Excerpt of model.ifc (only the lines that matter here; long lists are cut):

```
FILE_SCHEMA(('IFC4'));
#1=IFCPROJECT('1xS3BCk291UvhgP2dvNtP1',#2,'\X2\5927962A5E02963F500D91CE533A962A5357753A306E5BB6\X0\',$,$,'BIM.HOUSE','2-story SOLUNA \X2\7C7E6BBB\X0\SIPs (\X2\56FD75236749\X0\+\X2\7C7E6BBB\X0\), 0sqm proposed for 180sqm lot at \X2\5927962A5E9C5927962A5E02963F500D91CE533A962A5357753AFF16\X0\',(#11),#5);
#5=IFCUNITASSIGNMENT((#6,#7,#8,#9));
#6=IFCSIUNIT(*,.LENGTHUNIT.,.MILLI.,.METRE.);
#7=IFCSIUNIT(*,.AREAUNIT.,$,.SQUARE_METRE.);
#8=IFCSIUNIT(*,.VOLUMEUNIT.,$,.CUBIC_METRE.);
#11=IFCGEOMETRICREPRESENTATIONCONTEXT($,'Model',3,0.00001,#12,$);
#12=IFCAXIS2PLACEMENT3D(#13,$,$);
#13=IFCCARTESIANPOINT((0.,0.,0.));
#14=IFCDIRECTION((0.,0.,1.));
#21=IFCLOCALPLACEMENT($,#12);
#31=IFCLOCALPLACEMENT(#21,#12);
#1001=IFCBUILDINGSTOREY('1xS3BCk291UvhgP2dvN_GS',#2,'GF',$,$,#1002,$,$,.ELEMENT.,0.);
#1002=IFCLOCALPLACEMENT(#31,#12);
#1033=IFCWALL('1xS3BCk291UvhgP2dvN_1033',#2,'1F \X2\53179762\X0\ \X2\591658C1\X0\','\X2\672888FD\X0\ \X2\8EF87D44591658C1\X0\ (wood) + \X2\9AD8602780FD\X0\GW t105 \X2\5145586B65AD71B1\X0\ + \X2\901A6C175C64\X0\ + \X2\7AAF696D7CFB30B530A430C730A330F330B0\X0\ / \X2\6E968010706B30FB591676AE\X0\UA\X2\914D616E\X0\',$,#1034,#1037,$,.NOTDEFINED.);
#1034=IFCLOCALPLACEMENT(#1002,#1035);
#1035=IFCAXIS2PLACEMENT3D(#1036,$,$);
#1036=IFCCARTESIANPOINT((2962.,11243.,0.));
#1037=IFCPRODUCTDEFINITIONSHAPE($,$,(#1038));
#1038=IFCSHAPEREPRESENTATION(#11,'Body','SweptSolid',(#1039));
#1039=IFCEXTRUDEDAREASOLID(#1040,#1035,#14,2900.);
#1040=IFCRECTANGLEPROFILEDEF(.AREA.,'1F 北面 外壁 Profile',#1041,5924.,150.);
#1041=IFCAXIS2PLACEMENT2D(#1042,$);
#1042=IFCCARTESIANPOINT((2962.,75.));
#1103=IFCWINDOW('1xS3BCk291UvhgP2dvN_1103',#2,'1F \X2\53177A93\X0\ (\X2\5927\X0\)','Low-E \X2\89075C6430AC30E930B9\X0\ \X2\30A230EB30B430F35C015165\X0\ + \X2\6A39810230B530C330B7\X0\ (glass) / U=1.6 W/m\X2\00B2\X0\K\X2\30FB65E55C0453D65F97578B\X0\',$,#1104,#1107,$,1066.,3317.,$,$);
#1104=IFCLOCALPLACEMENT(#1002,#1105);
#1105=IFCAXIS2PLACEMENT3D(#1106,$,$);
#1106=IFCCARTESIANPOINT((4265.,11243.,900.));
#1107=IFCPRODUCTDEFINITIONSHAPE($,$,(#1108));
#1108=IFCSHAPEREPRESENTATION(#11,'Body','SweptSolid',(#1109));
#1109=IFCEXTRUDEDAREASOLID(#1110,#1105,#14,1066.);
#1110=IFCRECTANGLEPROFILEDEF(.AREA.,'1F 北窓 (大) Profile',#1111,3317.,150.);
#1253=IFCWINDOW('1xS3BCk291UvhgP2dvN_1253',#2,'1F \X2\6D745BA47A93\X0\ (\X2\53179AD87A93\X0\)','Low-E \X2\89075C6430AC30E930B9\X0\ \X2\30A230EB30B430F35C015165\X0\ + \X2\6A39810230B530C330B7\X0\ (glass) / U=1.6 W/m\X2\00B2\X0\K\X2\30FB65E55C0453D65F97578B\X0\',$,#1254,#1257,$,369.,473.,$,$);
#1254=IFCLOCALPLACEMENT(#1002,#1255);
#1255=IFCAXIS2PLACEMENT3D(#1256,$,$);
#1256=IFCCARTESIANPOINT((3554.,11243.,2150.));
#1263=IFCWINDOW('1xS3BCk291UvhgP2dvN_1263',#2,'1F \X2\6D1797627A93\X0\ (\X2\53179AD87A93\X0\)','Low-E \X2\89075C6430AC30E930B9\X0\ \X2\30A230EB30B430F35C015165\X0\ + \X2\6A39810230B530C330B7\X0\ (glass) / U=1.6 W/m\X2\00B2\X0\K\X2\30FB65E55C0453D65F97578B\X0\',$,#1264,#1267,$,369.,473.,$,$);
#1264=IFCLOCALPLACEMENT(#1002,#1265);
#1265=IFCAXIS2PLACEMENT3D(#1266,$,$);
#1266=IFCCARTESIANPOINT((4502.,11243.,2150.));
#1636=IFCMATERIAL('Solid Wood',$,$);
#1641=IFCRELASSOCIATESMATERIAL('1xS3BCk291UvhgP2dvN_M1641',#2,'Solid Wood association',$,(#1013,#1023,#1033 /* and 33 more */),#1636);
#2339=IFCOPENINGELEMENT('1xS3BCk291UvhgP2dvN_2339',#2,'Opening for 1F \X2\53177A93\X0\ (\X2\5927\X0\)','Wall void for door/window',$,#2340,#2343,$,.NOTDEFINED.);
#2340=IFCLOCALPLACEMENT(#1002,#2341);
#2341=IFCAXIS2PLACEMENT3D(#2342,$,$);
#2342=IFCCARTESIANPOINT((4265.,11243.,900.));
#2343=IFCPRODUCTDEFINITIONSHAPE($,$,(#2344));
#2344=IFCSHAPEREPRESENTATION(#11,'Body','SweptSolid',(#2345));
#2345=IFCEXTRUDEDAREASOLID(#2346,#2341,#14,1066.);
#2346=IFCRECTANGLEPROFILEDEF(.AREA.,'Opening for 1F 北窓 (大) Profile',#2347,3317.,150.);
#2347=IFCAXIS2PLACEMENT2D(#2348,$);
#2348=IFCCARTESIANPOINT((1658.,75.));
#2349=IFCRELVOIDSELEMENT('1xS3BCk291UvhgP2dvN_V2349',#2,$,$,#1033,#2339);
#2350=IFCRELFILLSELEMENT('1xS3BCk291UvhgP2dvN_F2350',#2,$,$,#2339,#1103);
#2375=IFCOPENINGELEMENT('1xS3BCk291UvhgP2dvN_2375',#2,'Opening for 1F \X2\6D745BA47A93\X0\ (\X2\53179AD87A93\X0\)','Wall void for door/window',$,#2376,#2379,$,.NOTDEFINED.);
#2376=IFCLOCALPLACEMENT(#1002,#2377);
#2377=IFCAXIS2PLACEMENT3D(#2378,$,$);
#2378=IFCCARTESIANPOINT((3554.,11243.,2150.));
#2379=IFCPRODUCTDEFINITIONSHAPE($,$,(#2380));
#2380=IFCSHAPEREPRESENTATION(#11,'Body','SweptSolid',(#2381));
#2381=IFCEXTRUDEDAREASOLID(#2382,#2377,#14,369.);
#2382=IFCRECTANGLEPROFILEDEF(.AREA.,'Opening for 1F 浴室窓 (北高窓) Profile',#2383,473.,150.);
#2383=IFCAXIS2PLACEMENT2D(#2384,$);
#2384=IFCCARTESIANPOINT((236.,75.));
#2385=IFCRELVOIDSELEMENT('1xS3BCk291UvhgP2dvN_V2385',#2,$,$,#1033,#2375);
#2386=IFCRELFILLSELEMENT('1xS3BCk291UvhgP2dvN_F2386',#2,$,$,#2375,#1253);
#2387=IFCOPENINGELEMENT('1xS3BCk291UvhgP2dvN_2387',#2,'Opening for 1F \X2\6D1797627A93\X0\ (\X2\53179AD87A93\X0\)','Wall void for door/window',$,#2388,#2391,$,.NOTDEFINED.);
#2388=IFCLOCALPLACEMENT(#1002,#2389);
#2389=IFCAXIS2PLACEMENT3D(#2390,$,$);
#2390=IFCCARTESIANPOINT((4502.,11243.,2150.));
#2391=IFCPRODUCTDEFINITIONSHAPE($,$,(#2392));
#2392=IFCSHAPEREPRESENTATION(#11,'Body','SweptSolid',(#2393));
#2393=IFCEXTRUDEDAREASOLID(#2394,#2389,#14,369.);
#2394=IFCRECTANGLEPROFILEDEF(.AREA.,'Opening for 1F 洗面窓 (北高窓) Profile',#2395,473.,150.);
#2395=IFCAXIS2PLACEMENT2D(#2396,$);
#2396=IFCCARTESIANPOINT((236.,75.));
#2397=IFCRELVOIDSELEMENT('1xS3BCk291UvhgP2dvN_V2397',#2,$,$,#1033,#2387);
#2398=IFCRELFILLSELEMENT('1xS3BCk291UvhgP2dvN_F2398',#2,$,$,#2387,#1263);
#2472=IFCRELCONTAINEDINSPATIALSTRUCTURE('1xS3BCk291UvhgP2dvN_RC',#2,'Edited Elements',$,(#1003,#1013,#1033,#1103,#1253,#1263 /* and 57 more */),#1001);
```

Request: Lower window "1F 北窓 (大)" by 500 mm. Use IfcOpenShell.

```python
import numpy as np
import ifcopenshell
import ifcopenshell.api.geometry
import ifcopenshell.util.placement
import ifcopenshell.util.unit

model = ifcopenshell.open("model.ifc")
unit_scale = ifcopenshell.util.unit.calculate_unit_scale(model)

window = model.by_guid("1xS3BCk291UvhgP2dvN_1103")
opening = window.FillsVoids[0].RelatingOpeningElement
dz = -0.5 / unit_scale

shift = np.array([0.0, 0.0, dz])
# The window is not placed relative to its opening, so move both.
for product in (opening, window):
    matrix = ifcopenshell.util.placement.get_local_placement(product.ObjectPlacement)
    matrix[:3, 3] += shift
    ifcopenshell.api.geometry.edit_object_placement(model, product=product, matrix=matrix, is_si=False)

print(f"moved by {dz * unit_scale:+.3f} m")

model.write("model_v2.ifc")
```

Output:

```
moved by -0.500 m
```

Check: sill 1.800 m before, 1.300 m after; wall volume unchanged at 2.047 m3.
